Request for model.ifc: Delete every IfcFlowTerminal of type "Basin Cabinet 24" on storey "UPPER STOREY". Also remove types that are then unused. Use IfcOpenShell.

First a look at what the model holds.

```python
import ifcopenshell
import ifcopenshell.util.element

model = ifcopenshell.open("model.ifc")
print(model.schema)
storey = next(s for s in model.by_type("IfcBuildingStorey") if s.Name == "UPPER STOREY")
terminals = [e for e in ifcopenshell.util.element.get_decomposition(storey) if e.is_a("IfcFlowTerminal")]
seen = {}
for e in terminals:
    element_type = ifcopenshell.util.element.get_type(e)
    name = element_type.Name if element_type not in (None, e) else None
    seen[name] = seen.get(name, 0) + 1
for name, count in sorted(seen.items(), key=str):
    print(count, "x", name)
```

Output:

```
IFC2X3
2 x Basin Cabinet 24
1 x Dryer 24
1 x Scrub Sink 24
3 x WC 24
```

```python
import ifcopenshell
import ifcopenshell.api.root
import ifcopenshell.util.element

model = ifcopenshell.open("model.ifc")

storey = next(s for s in model.by_type("IfcBuildingStorey") if s.Name == "UPPER STOREY")
terminals = [e for e in ifcopenshell.util.element.get_decomposition(storey) if e.is_a("IfcFlowTerminal")]
targets = [e for e in terminals if (t := ifcopenshell.util.element.get_type(e)) not in (None, e) and t.Name == "Basin Cabinet 24"]
types = {ifcopenshell.util.element.get_type(e) for e in targets} - {None, *targets}

for e in targets:
    ifcopenshell.api.root.remove_product(model, product=e)
print(len(targets), "removed")

unused = [t for t in types if not ifcopenshell.util.element.get_types(t)]
for t in unused:
    ifcopenshell.api.root.remove_product(model, product=t)
print(len(unused), "unused types removed")

model.write("model_updated.ifc")
```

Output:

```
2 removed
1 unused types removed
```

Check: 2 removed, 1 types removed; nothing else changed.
